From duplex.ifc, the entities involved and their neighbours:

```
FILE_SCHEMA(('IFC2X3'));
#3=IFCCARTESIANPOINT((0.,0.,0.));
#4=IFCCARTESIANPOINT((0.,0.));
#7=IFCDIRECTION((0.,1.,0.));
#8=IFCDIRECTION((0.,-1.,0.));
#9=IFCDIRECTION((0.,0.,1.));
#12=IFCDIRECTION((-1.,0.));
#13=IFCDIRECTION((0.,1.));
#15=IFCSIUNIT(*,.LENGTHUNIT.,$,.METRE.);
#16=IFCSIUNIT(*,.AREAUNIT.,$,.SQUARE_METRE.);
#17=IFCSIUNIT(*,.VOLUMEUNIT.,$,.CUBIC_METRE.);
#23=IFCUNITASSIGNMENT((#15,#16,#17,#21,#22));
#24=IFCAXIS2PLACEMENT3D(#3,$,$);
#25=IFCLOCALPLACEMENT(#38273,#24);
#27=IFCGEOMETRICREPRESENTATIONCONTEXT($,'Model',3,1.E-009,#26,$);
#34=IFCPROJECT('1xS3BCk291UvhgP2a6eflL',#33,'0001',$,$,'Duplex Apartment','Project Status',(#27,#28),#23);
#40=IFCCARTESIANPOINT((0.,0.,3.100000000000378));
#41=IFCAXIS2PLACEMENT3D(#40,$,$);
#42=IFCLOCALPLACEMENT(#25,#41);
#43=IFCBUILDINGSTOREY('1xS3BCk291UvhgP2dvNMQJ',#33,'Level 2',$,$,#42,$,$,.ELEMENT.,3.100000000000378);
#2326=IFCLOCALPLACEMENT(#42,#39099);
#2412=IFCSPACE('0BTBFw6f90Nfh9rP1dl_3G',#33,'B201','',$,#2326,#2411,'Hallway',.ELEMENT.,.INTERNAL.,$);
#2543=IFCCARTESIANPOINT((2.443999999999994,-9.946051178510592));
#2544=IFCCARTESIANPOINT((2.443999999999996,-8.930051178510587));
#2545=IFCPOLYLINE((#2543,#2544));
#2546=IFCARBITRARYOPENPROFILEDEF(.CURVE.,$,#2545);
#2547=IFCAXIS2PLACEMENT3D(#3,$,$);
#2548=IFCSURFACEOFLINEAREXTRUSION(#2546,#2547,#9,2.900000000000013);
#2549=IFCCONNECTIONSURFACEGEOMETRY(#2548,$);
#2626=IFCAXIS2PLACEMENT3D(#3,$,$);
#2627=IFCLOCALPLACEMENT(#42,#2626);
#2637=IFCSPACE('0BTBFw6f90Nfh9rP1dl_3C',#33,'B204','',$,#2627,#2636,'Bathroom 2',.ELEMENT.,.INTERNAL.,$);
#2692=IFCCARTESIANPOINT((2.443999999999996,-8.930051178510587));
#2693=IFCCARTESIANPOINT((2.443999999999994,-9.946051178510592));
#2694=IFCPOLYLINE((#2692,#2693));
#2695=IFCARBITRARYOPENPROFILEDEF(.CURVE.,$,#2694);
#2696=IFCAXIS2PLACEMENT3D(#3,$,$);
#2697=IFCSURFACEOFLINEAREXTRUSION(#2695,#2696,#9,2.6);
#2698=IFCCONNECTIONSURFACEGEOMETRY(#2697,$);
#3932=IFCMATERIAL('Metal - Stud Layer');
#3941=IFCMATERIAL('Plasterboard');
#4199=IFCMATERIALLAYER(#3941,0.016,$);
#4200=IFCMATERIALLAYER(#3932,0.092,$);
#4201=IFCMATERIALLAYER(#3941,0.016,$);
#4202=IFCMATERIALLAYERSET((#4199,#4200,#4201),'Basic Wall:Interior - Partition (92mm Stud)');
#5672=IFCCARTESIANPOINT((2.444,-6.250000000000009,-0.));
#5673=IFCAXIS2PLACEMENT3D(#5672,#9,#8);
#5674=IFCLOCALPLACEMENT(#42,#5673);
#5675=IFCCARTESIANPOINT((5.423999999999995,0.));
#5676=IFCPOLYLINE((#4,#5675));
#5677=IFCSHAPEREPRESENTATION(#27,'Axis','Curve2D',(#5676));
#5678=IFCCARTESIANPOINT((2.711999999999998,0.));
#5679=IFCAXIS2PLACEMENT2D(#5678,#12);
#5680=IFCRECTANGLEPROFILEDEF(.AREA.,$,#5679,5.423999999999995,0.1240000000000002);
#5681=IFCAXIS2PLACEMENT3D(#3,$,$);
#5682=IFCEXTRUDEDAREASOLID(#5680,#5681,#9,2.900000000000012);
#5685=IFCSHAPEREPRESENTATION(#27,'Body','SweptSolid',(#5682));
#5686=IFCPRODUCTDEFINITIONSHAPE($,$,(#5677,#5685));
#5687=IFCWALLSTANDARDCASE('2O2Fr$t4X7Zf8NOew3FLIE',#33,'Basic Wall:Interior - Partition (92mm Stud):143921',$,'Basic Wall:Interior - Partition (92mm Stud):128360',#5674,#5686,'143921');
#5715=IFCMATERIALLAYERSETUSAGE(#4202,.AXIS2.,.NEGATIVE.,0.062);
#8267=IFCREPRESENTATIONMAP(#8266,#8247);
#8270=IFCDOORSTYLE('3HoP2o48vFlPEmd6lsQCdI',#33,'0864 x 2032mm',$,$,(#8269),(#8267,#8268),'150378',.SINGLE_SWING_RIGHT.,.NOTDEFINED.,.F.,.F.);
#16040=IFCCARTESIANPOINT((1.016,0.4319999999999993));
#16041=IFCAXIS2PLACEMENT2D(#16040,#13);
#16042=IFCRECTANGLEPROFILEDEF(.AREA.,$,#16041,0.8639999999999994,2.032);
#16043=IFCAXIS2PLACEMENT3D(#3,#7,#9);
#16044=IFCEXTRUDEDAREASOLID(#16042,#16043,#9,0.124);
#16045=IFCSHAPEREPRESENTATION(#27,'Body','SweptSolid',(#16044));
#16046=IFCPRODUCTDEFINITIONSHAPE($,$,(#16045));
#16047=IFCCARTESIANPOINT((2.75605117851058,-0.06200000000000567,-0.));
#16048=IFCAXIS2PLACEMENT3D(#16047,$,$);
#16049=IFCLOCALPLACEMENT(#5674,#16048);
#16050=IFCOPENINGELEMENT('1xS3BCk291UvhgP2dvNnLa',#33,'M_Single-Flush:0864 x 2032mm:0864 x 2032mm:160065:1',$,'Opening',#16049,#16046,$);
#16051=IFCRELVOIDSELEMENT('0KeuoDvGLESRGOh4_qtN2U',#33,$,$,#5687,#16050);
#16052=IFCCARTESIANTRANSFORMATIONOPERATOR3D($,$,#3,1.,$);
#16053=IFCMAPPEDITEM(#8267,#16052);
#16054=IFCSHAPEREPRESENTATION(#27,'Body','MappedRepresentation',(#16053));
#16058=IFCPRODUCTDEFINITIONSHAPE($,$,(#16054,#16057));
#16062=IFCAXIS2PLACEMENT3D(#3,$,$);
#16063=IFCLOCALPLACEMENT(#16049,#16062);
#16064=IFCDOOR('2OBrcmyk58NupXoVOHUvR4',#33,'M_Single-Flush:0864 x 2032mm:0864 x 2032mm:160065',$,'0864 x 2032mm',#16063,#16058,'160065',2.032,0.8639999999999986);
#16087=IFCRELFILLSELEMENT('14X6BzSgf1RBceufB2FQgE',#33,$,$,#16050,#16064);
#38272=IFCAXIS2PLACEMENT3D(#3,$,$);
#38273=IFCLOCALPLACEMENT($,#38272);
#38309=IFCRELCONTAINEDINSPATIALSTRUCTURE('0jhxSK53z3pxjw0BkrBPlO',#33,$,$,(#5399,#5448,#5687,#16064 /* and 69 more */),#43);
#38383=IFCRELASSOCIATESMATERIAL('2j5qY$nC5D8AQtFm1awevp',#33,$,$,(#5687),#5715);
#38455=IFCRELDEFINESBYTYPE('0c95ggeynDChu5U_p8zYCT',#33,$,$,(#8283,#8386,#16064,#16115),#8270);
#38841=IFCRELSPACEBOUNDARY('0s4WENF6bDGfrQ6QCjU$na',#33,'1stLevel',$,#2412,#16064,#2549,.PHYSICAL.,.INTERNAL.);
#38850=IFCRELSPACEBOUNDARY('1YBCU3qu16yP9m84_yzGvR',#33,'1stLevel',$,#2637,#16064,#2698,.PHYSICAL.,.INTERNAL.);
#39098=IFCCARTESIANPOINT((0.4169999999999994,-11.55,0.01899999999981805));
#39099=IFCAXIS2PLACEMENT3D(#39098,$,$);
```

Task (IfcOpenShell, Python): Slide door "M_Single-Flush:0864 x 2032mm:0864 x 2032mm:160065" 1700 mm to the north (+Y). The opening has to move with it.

```python
import numpy as np
import ifcopenshell
import ifcopenshell.api.geometry
import ifcopenshell.util.placement
import ifcopenshell.util.unit

model = ifcopenshell.open("duplex.ifc")
unit_scale = ifcopenshell.util.unit.calculate_unit_scale(model)

door = model.by_id(16064)
opening = door.FillsVoids[0].RelatingOpeningElement
wall = opening.VoidsElements[0].RelatingBuildingElement

wall_matrix = ifcopenshell.util.placement.get_local_placement(wall.ObjectPlacement)
shift = wall_matrix[:3, 0] * -1.7 / unit_scale
before = ifcopenshell.util.placement.get_local_placement(door.ObjectPlacement)[:3, 3].copy()

# The door is placed relative to its opening, so it follows when the opening moves.
matrix = ifcopenshell.util.placement.get_local_placement(opening.ObjectPlacement)
matrix[:3, 3] += shift
ifcopenshell.api.geometry.edit_object_placement(
    model, product=opening, matrix=matrix, is_si=False, should_transform_children=True
)

# Space boundary surfaces are stored in each space's coordinates; move them too.
for rel in door.ProvidesBoundaries:
    if not rel.ConnectionGeometry:
        continue
    surface = rel.ConnectionGeometry.SurfaceOnRelatingElement
    space_matrix = ifcopenshell.util.placement.get_local_placement(rel.RelatingSpace.ObjectPlacement)
    point = np.array(surface.Position.Location.Coordinates) + space_matrix[:3, :3].T @ shift
    surface.Position = model.createIfcAxis2Placement3D(
        model.createIfcCartesianPoint(point.tolist()), surface.Position.Axis, surface.Position.RefDirection
    )

after = ifcopenshell.util.placement.get_local_placement(door.ObjectPlacement)[:3, 3]
print("door moved by", (after - before).round(3) + 0.0)

model.write("duplex_edited.ifc")
```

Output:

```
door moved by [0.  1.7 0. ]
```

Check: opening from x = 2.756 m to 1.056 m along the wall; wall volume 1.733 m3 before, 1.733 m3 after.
